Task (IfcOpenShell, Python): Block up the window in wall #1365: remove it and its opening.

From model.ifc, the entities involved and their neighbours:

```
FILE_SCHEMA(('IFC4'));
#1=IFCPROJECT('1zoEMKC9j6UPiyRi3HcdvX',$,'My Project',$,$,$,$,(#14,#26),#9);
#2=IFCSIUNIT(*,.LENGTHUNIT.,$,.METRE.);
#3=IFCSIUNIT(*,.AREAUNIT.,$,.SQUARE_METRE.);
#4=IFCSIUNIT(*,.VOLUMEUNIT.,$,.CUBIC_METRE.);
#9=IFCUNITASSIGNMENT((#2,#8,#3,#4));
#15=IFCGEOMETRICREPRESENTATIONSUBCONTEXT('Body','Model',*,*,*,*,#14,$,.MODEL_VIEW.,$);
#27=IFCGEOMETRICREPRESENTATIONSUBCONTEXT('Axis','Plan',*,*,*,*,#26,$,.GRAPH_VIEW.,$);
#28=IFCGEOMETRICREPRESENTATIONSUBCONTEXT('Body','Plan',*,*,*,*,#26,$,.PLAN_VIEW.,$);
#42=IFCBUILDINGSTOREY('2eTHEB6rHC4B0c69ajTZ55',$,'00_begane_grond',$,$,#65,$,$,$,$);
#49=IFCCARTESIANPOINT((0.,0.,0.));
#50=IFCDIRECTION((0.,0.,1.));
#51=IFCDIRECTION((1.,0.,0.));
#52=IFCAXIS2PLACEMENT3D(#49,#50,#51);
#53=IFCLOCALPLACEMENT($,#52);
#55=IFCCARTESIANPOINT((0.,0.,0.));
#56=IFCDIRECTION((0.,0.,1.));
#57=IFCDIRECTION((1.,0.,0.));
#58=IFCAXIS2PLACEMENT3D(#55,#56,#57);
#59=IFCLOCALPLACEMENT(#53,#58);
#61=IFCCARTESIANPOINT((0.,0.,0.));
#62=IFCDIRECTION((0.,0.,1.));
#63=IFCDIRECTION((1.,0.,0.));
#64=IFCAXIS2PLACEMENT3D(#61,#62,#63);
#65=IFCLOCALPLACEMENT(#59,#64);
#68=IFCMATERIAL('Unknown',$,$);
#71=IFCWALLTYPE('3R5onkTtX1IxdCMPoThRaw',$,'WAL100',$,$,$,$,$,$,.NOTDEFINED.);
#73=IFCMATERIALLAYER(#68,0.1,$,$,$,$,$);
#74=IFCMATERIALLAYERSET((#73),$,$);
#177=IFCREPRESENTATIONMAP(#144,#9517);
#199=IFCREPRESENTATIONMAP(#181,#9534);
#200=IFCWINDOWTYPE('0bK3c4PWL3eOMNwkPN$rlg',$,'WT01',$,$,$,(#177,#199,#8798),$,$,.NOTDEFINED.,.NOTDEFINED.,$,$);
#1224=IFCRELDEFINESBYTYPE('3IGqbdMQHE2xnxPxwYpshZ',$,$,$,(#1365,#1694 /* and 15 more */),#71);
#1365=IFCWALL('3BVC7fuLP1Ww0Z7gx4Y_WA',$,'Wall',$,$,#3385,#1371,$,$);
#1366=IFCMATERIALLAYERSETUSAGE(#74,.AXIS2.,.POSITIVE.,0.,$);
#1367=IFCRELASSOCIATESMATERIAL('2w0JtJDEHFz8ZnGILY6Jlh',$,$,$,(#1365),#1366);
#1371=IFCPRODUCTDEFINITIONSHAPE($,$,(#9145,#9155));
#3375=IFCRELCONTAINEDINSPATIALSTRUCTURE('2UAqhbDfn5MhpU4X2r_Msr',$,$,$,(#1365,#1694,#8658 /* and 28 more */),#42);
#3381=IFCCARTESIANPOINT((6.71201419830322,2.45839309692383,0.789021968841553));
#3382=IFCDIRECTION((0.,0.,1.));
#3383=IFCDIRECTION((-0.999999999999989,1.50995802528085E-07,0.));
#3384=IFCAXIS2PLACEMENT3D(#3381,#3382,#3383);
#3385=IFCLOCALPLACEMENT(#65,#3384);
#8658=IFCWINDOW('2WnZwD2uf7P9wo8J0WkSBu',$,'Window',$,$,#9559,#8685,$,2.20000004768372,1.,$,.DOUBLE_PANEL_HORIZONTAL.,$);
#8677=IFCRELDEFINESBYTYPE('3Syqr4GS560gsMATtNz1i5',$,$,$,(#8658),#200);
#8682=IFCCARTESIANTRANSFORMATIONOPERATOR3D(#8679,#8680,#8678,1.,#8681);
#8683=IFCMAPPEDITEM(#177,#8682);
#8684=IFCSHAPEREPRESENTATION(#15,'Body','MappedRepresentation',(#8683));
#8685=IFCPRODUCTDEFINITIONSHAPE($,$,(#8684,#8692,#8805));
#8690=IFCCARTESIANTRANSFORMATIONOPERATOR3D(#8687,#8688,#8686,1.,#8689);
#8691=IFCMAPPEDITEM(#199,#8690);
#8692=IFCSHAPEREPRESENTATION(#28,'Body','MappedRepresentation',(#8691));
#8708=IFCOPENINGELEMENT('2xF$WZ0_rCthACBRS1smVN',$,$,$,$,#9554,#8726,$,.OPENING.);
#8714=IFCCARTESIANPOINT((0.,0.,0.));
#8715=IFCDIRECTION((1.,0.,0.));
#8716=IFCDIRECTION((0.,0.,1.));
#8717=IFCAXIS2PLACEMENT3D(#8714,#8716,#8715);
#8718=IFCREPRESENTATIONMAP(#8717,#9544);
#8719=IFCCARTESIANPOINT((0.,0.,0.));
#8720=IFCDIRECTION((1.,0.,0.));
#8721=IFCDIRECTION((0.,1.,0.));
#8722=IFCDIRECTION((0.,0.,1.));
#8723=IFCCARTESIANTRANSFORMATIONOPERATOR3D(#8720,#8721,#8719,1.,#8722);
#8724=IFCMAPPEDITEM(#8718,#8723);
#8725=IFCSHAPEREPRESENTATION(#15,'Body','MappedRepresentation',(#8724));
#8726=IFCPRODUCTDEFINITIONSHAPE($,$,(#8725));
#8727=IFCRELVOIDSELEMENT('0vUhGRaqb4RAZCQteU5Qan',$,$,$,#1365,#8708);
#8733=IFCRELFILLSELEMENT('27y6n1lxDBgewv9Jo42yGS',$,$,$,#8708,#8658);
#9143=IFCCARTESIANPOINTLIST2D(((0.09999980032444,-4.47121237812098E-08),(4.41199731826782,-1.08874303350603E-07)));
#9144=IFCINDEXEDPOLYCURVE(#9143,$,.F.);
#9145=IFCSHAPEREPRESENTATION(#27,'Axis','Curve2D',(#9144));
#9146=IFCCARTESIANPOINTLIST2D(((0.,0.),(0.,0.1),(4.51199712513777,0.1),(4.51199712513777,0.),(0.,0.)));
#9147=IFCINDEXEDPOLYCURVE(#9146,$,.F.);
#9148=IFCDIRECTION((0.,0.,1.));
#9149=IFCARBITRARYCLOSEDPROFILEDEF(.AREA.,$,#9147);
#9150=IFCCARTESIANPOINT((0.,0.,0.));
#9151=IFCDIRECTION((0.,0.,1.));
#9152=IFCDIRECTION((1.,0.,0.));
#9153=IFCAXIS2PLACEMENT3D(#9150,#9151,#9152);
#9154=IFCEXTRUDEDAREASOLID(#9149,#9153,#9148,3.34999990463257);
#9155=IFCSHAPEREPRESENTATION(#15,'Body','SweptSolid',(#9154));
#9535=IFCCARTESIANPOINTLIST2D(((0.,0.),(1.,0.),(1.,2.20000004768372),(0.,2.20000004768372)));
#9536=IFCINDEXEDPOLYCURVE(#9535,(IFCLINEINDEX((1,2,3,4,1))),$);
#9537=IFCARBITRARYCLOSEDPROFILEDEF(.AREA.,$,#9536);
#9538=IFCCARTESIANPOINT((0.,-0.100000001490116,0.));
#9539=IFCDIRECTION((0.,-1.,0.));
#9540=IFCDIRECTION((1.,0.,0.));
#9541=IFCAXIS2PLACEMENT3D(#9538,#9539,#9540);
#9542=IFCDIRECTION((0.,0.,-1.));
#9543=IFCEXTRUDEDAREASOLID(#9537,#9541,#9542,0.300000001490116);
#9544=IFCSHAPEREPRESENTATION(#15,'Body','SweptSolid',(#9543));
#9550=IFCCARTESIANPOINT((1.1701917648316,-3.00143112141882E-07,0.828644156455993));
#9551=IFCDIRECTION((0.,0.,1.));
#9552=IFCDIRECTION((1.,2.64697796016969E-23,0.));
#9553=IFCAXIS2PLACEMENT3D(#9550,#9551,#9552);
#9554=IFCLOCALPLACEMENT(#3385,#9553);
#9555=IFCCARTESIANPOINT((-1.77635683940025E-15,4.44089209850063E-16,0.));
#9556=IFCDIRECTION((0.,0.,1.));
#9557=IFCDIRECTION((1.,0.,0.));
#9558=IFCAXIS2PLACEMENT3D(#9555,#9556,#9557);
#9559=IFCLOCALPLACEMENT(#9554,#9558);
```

```python
import ifcopenshell
import ifcopenshell.api.feature
import ifcopenshell.api.root
import ifcopenshell.geom
import ifcopenshell.util.shape

model = ifcopenshell.open("model.ifc")
settings = ifcopenshell.geom.settings()


def volume(element):
    """Net volume in cubic metres, openings subtracted."""
    shape = ifcopenshell.geom.create_shape(settings, element)
    return ifcopenshell.util.shape.get_volume(shape.geometry)


window = model.by_guid("2WnZwD2uf7P9wo8J0WkSBu")
opening = window.FillsVoids[0].RelatingOpeningElement
wall = opening.VoidsElements[0].RelatingBuildingElement
before = volume(wall)

ifcopenshell.api.root.remove_product(model, product=window)
ifcopenshell.api.feature.remove_feature(model, feature=opening)

after = volume(wall)

print(f"wall volume {before:.3f} -> {after:.3f} m3")

model.write("model_rev.ifc")
```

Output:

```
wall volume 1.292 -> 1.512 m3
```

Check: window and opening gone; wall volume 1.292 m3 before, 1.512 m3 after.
